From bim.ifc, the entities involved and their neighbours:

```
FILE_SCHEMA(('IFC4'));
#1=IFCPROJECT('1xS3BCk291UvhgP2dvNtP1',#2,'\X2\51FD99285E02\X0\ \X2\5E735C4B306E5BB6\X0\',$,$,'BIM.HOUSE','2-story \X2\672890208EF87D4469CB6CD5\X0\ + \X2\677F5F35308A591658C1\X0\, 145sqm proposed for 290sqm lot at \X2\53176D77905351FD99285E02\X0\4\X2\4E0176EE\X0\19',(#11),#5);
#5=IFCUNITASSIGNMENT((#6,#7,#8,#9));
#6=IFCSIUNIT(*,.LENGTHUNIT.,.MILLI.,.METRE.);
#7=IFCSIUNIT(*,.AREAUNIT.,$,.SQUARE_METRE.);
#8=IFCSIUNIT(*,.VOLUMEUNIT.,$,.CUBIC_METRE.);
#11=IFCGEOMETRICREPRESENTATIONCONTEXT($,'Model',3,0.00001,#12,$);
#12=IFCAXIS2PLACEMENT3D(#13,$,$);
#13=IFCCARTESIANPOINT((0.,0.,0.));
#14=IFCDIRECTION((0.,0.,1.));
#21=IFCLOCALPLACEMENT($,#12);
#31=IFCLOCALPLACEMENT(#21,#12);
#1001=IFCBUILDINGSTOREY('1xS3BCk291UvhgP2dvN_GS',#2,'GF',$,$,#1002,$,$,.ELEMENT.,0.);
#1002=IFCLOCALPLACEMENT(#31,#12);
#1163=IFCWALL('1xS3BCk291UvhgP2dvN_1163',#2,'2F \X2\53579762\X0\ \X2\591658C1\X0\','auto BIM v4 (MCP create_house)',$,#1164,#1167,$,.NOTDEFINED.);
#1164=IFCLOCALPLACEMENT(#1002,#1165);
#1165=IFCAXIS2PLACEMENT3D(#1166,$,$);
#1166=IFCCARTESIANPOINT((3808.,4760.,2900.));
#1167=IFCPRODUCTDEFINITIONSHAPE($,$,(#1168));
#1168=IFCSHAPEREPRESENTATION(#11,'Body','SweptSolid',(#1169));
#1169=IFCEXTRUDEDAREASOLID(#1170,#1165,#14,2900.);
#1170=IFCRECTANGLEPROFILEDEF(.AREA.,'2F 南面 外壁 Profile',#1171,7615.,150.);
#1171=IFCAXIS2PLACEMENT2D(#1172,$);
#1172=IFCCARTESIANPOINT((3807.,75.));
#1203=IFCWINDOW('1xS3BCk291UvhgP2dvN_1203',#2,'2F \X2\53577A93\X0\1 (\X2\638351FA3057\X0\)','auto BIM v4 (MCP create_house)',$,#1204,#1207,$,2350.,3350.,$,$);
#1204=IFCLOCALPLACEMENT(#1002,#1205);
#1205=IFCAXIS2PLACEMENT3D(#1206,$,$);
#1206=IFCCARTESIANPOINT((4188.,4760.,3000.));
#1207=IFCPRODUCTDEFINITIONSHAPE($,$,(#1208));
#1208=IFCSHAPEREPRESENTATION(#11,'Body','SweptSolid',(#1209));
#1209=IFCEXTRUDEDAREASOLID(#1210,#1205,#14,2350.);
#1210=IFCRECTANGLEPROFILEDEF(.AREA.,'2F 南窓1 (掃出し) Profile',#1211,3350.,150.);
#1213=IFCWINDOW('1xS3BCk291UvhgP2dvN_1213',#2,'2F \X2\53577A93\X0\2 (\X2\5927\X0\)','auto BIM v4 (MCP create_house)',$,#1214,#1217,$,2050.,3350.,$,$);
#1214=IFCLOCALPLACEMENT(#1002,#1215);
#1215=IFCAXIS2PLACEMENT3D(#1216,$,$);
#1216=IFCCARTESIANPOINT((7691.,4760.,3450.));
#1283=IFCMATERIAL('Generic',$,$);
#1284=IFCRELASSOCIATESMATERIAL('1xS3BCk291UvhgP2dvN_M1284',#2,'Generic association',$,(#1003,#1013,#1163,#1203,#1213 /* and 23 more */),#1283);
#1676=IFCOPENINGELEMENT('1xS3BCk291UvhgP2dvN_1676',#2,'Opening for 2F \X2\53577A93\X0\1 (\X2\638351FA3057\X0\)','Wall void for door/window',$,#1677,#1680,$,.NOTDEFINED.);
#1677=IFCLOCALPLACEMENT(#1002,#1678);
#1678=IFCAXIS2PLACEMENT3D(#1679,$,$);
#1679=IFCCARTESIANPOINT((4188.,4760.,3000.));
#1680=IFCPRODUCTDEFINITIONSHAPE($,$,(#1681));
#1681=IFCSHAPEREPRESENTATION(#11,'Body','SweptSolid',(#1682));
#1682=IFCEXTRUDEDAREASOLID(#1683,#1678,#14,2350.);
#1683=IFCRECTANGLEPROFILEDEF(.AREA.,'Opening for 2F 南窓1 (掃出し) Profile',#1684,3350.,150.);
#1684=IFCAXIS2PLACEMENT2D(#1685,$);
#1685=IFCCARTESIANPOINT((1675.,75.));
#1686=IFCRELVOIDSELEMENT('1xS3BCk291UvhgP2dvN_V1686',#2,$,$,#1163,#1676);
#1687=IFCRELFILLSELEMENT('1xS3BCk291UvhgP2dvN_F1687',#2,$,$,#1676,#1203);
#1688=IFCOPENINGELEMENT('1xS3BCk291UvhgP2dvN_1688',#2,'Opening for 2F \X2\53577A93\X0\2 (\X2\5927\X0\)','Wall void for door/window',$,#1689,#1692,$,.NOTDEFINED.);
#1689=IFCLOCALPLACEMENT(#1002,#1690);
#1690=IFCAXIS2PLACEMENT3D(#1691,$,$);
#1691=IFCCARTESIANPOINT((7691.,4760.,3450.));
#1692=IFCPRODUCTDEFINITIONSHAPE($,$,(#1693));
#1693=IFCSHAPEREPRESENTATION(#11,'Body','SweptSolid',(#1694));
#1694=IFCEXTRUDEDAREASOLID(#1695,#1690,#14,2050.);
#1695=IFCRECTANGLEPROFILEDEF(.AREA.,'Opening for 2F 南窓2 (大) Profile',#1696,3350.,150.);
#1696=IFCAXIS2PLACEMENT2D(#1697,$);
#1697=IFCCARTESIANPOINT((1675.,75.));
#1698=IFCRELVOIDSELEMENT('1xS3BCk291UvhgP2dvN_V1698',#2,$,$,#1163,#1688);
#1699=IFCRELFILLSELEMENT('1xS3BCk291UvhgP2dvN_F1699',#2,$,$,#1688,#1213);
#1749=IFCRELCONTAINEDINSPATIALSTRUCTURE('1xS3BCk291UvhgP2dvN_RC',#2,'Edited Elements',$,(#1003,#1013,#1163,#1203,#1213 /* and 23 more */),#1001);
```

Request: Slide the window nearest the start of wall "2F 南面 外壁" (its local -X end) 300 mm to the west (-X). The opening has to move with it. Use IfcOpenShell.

```python
import ifcopenshell
import ifcopenshell.api.geometry
import ifcopenshell.util.placement
import ifcopenshell.util.unit

model = ifcopenshell.open("bim.ifc")
unit_scale = ifcopenshell.util.unit.calculate_unit_scale(model)

window = model.by_guid("1xS3BCk291UvhgP2dvN_1203")
opening = window.FillsVoids[0].RelatingOpeningElement
wall = opening.VoidsElements[0].RelatingBuildingElement

wall_matrix = ifcopenshell.util.placement.get_local_placement(wall.ObjectPlacement)
shift = wall_matrix[:3, 0] * -0.3 / unit_scale
before = ifcopenshell.util.placement.get_local_placement(window.ObjectPlacement)[:3, 3].copy()

# The window is not placed relative to its opening, so move both.
for product in (opening, window):
    matrix = ifcopenshell.util.placement.get_local_placement(product.ObjectPlacement)
    matrix[:3, 3] += shift
    ifcopenshell.api.geometry.edit_object_placement(model, product=product, matrix=matrix, is_si=False)

after = ifcopenshell.util.placement.get_local_placement(window.ObjectPlacement)[:3, 3]
print("window moved by", (after - before).round(3) + 0.0)

model.write("bim_updated.ifc")
```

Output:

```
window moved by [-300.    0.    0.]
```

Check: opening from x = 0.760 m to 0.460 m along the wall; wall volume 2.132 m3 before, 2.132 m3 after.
